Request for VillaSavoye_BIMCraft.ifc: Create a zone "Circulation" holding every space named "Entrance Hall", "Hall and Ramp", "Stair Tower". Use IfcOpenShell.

First a look at what the model holds.

```python
import ifcopenshell

model = ifcopenshell.open("VillaSavoye_BIMCraft.ifc")
print(model.schema)
seen = {}
for space in model.by_type("IfcSpace"):
    seen[space.LongName] = seen.get(space.LongName, 0) + 1
for name, count in sorted(seen.items(), key=str):
    print(count, "x", name)
print("zones:", [z.Name for z in model.by_type("IfcZone")][:20])
```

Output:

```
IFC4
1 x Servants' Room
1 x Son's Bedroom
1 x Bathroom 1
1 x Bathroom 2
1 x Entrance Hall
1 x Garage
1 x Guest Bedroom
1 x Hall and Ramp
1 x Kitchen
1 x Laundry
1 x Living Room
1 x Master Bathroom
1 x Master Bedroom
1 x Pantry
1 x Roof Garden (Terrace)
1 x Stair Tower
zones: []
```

```python
import ifcopenshell
import ifcopenshell.api.group
import ifcopenshell.api.root

model = ifcopenshell.open("VillaSavoye_BIMCraft.ifc")

names = {"Entrance Hall", "Hall and Ramp", "Stair Tower"}
spaces = [s for s in model.by_type("IfcSpace") if s.LongName in names]

zone = ifcopenshell.api.root.create_entity(model, ifc_class="IfcZone", name="Circulation")
ifcopenshell.api.group.assign_group(model, products=spaces, group=zone)
print(len(spaces), "spaces in", zone.Name)

model.write("VillaSavoye_BIMCraft_v2.ifc")
```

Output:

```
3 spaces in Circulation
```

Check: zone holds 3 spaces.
